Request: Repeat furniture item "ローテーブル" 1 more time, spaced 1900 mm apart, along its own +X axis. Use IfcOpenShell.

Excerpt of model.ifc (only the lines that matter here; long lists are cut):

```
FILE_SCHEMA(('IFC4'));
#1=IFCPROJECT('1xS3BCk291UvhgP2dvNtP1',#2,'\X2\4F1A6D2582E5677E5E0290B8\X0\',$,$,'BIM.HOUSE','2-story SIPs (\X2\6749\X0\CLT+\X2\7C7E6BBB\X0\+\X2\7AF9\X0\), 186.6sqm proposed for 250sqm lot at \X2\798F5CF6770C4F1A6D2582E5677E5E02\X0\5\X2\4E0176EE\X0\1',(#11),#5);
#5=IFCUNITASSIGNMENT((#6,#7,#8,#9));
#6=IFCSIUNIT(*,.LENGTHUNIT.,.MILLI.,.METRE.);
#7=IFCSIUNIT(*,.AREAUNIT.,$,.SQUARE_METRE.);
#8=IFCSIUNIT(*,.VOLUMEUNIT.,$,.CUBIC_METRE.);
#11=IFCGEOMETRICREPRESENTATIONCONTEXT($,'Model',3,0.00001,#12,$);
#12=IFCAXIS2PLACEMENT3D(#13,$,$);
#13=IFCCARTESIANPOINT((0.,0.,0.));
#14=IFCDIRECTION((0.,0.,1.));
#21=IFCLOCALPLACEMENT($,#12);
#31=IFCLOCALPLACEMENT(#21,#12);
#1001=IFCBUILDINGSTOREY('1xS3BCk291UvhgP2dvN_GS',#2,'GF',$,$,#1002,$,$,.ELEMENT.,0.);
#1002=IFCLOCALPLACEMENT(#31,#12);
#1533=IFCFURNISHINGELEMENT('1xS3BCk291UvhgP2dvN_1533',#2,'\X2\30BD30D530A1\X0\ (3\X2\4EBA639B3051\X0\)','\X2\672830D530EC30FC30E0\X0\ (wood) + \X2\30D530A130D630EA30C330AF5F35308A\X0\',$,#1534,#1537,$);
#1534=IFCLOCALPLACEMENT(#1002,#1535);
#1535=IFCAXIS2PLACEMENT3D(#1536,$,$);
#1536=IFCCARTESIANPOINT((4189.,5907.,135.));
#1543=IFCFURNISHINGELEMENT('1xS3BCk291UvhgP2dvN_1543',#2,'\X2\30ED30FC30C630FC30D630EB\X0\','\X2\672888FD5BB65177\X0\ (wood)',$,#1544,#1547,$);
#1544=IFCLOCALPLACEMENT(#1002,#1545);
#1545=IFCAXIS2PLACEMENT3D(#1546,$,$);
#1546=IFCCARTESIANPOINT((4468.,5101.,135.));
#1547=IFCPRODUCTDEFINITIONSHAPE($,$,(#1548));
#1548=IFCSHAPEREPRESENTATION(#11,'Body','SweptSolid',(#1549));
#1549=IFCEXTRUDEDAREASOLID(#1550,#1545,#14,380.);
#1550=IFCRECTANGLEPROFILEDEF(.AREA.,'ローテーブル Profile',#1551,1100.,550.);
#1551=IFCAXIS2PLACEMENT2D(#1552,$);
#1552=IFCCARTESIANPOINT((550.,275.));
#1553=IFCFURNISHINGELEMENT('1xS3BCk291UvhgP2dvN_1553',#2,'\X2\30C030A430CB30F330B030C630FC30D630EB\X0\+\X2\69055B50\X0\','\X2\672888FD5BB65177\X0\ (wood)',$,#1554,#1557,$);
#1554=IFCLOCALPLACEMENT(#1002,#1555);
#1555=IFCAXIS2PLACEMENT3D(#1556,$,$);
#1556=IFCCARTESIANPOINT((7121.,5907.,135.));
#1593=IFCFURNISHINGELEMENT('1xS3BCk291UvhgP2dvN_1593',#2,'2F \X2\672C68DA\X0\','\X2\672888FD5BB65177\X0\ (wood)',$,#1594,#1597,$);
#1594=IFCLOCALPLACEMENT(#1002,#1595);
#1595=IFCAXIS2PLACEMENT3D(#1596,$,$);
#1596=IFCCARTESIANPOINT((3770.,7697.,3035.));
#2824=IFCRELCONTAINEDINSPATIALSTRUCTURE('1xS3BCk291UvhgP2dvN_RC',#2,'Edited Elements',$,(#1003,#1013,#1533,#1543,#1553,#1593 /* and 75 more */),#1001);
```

```python
import ifcopenshell
import ifcopenshell.api.geometry
import ifcopenshell.api.root
import ifcopenshell.util.element
import ifcopenshell.util.placement

model = ifcopenshell.open("model.ifc")


def reuse_history(source, copy):
    """copy_class also copies each property set's owner history, people and application; keep the originals."""
    for rel in copy.IsDefinedBy:
        if rel.is_a("IfcRelDefinesByProperties") and (history := rel.RelatingPropertyDefinition.OwnerHistory):
            rel.RelatingPropertyDefinition.OwnerHistory = source.OwnerHistory
            ifcopenshell.util.element.remove_deep2(model, history)


source = model.by_guid("1xS3BCk291UvhgP2dvN_1543")
base = ifcopenshell.util.placement.get_local_placement(source.ObjectPlacement)
step = base[:3, 0] * 1900.0

for i in range(1, 2):
    copy = ifcopenshell.api.root.copy_class(model, product=source)
    copy.Representation = ifcopenshell.util.element.copy_deep(
        model, source.Representation, exclude=["IfcGeometricRepresentationContext", "IfcRepresentationMap"]
    )
    reuse_history(source, copy)
    matrix = base.copy()
    matrix[:3, 3] += i * step
    print("added at", matrix[:3, 3].round(3) + 0.0)
    ifcopenshell.api.geometry.edit_object_placement(model, product=copy, matrix=matrix, is_si=False)

model.write("model_rev.ifc")
```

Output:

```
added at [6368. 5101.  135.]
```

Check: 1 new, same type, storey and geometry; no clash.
